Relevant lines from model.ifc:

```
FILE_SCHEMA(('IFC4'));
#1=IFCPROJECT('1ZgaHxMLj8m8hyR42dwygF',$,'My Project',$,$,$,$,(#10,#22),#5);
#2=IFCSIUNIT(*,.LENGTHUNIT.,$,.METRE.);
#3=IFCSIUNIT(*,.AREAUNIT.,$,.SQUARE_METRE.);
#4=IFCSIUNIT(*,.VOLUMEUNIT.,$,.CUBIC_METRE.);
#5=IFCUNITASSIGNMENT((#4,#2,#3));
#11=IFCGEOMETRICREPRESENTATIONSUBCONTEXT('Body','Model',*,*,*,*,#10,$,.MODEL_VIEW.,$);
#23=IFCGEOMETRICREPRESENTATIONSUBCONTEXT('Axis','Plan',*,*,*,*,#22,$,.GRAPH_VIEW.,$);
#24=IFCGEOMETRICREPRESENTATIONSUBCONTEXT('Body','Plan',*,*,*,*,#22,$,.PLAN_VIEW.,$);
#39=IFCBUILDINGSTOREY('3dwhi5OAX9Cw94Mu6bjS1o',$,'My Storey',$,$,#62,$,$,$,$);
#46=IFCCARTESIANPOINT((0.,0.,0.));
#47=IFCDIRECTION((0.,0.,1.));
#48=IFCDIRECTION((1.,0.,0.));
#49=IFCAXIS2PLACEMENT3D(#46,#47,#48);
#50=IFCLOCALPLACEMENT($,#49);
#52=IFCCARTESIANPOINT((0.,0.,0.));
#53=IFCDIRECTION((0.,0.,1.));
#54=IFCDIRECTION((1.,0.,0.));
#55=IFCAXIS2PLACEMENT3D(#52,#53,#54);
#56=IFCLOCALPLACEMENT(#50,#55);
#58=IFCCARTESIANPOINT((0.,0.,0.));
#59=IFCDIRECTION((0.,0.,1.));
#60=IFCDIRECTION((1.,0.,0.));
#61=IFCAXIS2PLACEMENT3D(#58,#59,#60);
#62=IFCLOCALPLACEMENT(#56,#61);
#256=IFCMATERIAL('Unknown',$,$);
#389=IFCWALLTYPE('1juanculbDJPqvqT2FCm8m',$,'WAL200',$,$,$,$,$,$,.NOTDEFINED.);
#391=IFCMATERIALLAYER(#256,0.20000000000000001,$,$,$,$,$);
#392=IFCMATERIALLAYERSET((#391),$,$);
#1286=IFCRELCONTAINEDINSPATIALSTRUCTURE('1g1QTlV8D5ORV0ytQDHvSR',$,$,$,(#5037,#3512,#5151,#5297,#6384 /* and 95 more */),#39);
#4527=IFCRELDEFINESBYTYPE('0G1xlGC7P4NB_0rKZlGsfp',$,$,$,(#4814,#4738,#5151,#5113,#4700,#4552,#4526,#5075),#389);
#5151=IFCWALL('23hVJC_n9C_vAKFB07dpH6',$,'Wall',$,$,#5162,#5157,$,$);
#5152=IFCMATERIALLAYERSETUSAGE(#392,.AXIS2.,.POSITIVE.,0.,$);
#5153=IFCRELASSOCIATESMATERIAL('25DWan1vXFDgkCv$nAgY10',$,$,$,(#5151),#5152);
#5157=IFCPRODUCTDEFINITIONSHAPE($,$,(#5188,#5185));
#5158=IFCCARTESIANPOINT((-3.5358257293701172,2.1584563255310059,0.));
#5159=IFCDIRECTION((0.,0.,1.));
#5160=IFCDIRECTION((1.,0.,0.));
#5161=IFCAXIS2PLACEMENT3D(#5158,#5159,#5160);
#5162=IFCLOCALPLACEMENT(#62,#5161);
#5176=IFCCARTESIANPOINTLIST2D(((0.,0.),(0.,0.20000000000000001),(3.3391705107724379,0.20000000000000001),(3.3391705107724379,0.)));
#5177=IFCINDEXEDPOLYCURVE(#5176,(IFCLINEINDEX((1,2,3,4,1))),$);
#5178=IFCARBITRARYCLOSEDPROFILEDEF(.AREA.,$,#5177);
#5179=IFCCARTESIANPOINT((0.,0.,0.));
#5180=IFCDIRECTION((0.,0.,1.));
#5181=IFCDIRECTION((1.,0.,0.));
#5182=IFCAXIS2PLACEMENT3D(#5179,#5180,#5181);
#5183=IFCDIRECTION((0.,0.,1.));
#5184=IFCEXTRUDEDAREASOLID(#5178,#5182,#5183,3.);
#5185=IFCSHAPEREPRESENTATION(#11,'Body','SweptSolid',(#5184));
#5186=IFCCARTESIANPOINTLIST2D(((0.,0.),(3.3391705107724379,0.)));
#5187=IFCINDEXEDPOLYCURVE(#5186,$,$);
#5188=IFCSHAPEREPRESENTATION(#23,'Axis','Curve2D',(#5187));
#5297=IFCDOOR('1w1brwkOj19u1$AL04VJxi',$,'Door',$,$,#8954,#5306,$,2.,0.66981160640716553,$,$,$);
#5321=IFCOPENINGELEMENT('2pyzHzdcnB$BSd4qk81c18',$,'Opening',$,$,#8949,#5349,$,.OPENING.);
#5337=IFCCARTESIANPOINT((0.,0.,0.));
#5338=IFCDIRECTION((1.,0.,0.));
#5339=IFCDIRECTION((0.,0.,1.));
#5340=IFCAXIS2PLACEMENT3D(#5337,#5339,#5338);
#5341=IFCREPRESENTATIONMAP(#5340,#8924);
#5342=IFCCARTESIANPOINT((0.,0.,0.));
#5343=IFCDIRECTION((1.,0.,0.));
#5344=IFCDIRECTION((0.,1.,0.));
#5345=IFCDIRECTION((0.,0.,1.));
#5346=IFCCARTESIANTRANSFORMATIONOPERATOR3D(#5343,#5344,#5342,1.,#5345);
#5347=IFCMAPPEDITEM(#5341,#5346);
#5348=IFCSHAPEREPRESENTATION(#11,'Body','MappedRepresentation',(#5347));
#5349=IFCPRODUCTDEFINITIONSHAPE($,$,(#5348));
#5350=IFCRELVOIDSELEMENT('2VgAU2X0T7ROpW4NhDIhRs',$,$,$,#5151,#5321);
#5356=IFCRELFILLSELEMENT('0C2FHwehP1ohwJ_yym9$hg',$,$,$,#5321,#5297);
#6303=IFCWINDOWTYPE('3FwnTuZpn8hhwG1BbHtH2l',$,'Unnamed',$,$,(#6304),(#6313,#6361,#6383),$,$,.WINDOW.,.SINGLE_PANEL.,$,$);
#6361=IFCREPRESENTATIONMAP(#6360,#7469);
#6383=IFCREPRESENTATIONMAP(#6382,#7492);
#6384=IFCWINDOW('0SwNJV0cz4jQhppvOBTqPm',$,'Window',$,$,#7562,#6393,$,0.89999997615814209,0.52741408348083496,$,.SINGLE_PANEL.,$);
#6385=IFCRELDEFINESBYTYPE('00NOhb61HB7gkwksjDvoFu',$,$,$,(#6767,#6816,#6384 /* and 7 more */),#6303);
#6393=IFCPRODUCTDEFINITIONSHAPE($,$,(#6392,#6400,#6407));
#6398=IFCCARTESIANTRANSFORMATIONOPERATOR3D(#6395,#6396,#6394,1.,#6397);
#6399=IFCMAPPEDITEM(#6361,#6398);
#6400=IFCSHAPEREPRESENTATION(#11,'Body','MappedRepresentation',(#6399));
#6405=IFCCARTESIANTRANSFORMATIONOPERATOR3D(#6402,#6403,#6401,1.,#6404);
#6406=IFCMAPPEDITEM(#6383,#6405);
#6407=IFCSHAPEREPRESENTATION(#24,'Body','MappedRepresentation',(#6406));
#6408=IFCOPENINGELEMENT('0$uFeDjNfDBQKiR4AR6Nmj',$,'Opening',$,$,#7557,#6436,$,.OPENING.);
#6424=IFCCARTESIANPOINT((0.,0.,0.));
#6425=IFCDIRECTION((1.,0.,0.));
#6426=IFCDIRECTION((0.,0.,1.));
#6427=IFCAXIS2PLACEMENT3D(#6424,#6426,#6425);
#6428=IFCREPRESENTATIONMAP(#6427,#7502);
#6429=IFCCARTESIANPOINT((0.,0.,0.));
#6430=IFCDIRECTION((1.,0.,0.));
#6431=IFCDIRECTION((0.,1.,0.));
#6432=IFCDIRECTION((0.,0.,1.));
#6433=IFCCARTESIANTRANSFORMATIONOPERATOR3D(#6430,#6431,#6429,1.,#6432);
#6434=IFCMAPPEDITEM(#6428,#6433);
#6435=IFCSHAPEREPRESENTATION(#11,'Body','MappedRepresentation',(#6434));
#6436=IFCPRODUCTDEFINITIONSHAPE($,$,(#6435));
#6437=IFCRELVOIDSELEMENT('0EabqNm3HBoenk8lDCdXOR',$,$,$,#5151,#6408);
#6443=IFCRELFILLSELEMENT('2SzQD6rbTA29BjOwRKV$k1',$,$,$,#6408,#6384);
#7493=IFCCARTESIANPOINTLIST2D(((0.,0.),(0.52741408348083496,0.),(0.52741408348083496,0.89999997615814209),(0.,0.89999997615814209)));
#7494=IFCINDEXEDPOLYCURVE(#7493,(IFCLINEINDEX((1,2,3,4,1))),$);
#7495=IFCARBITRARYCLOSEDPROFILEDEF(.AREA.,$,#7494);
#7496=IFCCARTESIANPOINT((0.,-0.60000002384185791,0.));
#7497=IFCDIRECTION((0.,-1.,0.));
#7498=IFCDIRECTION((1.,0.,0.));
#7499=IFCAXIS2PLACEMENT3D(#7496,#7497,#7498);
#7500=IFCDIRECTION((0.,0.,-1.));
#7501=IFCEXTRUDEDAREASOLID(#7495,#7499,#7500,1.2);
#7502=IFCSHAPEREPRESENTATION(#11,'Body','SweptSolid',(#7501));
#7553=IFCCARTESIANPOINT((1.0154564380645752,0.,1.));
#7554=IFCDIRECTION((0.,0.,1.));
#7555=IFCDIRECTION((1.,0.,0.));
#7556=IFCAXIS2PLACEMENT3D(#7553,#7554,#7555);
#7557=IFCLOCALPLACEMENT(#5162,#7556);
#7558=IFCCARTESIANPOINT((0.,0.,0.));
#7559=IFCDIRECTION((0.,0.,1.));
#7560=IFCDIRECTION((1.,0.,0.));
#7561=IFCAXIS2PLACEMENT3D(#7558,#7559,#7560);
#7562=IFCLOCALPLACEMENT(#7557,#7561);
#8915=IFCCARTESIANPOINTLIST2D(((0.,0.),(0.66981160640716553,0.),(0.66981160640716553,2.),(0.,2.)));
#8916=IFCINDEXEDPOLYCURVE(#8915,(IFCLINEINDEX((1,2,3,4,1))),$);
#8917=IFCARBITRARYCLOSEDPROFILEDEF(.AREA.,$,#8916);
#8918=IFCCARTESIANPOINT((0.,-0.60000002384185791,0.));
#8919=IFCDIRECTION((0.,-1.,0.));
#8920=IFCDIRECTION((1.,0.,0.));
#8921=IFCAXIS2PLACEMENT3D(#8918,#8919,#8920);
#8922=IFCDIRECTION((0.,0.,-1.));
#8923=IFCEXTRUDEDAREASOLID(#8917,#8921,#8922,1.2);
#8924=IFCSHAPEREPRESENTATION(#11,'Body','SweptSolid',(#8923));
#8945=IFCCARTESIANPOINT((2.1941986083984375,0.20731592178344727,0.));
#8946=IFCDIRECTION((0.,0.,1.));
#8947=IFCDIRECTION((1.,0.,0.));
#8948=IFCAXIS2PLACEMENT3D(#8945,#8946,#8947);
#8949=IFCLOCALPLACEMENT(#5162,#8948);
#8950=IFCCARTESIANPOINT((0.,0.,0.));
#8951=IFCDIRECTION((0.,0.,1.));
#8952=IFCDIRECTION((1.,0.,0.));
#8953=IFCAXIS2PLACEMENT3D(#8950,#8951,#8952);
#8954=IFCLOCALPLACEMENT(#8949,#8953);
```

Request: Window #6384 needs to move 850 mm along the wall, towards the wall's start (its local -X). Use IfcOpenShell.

```python
import ifcopenshell
import ifcopenshell.api.geometry
import ifcopenshell.util.placement
import ifcopenshell.util.unit

model = ifcopenshell.open("model.ifc")
unit_scale = ifcopenshell.util.unit.calculate_unit_scale(model)

window = model.by_guid("0SwNJV0cz4jQhppvOBTqPm")
opening = window.FillsVoids[0].RelatingOpeningElement
wall = opening.VoidsElements[0].RelatingBuildingElement

wall_matrix = ifcopenshell.util.placement.get_local_placement(wall.ObjectPlacement)
shift = wall_matrix[:3, 0] * -0.85 / unit_scale
before = ifcopenshell.util.placement.get_local_placement(window.ObjectPlacement)[:3, 3].copy()

# The window is placed relative to its opening, so it follows when the opening moves.
matrix = ifcopenshell.util.placement.get_local_placement(opening.ObjectPlacement)
matrix[:3, 3] += shift
ifcopenshell.api.geometry.edit_object_placement(
    model, product=opening, matrix=matrix, is_si=False, should_transform_children=True
)

after = ifcopenshell.util.placement.get_local_placement(window.ObjectPlacement)[:3, 3]
print("window moved by", (after - before).round(3) + 0.0)

model.write("model_edited.ifc")
```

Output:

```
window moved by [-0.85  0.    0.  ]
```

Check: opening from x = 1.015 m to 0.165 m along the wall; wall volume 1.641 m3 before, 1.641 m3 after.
